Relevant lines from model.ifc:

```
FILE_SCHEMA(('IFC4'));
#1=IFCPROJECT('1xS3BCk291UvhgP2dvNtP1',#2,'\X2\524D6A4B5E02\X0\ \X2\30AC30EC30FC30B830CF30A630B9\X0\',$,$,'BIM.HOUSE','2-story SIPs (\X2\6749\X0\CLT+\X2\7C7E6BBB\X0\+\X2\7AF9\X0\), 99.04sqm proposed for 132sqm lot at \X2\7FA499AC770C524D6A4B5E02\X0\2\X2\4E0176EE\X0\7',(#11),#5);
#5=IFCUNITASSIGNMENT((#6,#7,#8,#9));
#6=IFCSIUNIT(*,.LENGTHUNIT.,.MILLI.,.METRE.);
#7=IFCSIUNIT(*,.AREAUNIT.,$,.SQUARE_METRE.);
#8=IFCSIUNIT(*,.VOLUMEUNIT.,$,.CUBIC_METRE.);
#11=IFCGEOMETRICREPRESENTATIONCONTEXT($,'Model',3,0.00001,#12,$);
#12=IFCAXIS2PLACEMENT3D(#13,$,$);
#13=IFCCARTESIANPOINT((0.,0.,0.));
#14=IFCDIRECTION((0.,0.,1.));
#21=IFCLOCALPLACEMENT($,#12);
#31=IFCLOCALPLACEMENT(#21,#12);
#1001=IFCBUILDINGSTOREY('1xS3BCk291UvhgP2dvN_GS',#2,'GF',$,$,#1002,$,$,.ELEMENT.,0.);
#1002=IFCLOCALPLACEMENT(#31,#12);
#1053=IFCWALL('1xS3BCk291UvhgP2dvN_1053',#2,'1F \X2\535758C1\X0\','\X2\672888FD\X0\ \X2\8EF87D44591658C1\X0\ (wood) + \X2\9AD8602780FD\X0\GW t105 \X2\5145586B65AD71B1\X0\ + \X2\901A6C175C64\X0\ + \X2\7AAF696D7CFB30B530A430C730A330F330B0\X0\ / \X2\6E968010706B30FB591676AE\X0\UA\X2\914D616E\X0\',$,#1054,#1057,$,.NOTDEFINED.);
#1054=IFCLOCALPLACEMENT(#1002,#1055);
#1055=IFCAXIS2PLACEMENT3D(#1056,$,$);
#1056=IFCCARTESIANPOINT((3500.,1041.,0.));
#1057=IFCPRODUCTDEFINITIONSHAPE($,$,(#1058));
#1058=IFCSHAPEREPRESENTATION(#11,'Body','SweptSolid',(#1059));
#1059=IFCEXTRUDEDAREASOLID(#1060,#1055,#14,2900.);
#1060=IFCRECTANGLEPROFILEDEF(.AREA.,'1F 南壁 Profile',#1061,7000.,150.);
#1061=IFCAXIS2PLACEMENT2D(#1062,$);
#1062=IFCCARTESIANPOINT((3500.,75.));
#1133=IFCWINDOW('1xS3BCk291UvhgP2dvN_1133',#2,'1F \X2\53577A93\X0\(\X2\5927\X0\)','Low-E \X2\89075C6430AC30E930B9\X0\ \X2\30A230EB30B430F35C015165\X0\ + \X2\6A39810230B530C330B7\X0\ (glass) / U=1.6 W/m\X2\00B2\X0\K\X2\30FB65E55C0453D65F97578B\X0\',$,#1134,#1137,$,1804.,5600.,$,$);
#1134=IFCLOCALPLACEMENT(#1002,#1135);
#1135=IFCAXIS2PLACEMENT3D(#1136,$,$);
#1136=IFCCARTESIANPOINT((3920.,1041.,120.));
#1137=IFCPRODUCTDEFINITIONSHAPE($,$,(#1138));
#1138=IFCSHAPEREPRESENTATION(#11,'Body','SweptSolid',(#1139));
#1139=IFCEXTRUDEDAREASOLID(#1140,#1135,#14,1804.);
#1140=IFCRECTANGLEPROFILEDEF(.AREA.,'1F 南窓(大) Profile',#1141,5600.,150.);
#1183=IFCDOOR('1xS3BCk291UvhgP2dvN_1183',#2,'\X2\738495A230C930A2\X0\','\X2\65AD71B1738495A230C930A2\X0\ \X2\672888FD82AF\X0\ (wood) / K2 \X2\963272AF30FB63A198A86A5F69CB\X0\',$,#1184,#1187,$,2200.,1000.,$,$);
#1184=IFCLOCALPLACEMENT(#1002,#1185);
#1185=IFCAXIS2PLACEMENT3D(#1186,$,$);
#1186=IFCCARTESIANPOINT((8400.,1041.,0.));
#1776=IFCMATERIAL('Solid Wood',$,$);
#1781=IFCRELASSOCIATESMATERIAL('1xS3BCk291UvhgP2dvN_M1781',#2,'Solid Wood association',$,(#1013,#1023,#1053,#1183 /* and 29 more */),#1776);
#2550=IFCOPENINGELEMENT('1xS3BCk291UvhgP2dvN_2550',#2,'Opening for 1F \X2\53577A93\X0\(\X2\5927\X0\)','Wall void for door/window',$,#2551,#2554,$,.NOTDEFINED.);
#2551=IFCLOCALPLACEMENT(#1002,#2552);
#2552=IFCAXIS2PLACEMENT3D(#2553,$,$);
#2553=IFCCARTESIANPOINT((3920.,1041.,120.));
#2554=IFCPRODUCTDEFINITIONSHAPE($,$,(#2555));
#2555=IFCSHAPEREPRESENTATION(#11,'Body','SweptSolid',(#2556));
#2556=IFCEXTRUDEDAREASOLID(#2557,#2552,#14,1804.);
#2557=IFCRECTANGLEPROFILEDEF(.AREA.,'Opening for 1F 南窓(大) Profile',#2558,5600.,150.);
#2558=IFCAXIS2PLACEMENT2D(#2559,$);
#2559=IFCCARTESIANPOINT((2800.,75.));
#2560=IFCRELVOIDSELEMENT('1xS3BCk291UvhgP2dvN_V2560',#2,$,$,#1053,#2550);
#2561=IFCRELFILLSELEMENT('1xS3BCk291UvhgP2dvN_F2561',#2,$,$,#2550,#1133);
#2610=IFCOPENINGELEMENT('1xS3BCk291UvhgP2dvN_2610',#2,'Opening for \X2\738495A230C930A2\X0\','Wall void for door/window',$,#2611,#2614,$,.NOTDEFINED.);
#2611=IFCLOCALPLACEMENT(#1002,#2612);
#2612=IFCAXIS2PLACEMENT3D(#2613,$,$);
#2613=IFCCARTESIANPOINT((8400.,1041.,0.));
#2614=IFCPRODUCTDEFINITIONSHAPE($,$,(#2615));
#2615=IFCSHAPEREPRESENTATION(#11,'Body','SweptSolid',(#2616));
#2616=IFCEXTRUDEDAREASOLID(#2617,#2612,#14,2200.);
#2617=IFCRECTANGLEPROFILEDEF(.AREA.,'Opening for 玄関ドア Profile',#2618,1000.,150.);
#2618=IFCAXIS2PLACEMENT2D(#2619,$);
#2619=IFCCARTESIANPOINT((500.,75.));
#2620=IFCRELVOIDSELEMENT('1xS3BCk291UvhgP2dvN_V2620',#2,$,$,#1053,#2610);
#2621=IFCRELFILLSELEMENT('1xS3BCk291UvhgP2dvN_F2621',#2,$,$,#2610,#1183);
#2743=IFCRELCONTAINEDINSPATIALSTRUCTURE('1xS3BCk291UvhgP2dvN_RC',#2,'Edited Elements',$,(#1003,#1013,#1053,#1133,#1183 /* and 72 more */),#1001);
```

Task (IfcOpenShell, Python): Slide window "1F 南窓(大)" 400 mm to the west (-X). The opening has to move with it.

```python
import ifcopenshell
import ifcopenshell.api.geometry
import ifcopenshell.util.placement

model = ifcopenshell.open("model.ifc")

window = model.by_guid("1xS3BCk291UvhgP2dvN_1133")
opening = window.FillsVoids[0].RelatingOpeningElement
wall = opening.VoidsElements[0].RelatingBuildingElement

wall_matrix = ifcopenshell.util.placement.get_local_placement(wall.ObjectPlacement)
shift = wall_matrix[:3, 0] * -400.0
before = ifcopenshell.util.placement.get_local_placement(window.ObjectPlacement)[:3, 3].copy()

# The window is not placed relative to its opening, so move both.
for product in (opening, window):
    matrix = ifcopenshell.util.placement.get_local_placement(product.ObjectPlacement)
    matrix[:3, 3] += shift
    ifcopenshell.api.geometry.edit_object_placement(model, product=product, matrix=matrix, is_si=False)

after = ifcopenshell.util.placement.get_local_placement(window.ObjectPlacement)[:3, 3]
print("window moved by", (after - before).round(3) + 0.0)

model.write("model_edited.ifc")
```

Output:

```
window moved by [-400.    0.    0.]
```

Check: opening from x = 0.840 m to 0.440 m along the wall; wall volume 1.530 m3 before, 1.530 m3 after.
